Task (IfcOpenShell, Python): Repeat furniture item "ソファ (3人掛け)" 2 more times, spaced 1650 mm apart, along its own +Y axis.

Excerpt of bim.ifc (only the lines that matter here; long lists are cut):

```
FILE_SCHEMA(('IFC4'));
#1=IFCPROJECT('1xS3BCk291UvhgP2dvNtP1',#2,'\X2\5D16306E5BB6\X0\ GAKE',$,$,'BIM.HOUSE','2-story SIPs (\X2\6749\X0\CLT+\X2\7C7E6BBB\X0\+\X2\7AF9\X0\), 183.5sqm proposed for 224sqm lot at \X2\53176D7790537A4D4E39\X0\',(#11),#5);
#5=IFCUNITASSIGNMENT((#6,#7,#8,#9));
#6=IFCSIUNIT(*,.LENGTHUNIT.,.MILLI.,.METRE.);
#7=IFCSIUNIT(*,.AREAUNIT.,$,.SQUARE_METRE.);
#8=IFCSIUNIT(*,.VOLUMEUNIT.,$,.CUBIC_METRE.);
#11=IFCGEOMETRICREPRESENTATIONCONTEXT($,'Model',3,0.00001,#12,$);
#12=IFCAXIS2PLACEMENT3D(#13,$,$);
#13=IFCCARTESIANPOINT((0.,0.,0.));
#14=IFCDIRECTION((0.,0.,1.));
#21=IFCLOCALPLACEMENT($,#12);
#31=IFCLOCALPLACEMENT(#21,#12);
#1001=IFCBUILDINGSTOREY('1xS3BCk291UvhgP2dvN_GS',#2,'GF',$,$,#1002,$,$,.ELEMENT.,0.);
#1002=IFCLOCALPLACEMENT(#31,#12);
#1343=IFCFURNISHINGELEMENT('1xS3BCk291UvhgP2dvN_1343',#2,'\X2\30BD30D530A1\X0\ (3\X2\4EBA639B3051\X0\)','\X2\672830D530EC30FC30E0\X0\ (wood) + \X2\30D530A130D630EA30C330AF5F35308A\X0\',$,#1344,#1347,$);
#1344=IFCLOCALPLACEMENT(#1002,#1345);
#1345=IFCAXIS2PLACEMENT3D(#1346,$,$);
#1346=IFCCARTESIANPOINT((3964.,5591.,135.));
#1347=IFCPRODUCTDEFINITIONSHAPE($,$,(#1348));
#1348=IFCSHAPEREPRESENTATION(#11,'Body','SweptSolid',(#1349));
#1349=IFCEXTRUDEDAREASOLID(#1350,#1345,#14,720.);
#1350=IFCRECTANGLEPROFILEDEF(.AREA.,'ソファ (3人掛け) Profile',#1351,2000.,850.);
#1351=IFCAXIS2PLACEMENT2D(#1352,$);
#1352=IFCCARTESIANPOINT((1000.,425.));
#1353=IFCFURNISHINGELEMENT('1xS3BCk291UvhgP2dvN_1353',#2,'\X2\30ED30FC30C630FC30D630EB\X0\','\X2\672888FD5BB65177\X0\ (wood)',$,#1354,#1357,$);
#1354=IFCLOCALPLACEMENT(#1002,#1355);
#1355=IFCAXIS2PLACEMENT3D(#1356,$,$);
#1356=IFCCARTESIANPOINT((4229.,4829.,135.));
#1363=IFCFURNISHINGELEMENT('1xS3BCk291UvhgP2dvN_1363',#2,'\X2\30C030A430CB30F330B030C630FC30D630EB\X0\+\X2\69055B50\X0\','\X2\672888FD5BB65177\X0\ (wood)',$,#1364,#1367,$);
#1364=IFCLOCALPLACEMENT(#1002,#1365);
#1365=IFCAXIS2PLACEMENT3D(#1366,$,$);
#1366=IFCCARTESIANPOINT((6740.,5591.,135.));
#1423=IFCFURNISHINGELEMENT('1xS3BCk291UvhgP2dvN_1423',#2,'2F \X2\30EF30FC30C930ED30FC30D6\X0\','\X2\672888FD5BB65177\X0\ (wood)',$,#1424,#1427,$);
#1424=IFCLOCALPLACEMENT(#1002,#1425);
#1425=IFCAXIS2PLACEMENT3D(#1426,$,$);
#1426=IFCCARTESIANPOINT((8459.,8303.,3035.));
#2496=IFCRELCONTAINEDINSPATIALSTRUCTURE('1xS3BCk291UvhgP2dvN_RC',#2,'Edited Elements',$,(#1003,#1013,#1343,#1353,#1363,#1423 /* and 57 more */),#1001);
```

```python
import ifcopenshell
import ifcopenshell.api.geometry
import ifcopenshell.api.root
import ifcopenshell.util.element
import ifcopenshell.util.placement
import ifcopenshell.util.unit

model = ifcopenshell.open("bim.ifc")
unit_scale = ifcopenshell.util.unit.calculate_unit_scale(model)


def reuse_history(source, copy):
    """copy_class also copies each property set's owner history, people and application; keep the originals."""
    for rel in copy.IsDefinedBy:
        if rel.is_a("IfcRelDefinesByProperties") and (history := rel.RelatingPropertyDefinition.OwnerHistory):
            rel.RelatingPropertyDefinition.OwnerHistory = source.OwnerHistory
            ifcopenshell.util.element.remove_deep2(model, history)


source = model.by_id(1343)
base = ifcopenshell.util.placement.get_local_placement(source.ObjectPlacement)
step = base[:3, 1] * 1.65 / unit_scale

for i in range(1, 3):
    copy = ifcopenshell.api.root.copy_class(model, product=source)
    copy.Representation = ifcopenshell.util.element.copy_deep(
        model, source.Representation, exclude=["IfcGeometricRepresentationContext", "IfcRepresentationMap"]
    )
    reuse_history(source, copy)
    matrix = base.copy()
    matrix[:3, 3] += i * step
    print("added at", matrix[:3, 3].round(3) + 0.0)
    ifcopenshell.api.geometry.edit_object_placement(model, product=copy, matrix=matrix, is_si=False)

model.write("bim_rev.ifc")
```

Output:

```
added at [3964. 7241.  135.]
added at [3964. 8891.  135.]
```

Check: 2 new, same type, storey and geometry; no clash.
